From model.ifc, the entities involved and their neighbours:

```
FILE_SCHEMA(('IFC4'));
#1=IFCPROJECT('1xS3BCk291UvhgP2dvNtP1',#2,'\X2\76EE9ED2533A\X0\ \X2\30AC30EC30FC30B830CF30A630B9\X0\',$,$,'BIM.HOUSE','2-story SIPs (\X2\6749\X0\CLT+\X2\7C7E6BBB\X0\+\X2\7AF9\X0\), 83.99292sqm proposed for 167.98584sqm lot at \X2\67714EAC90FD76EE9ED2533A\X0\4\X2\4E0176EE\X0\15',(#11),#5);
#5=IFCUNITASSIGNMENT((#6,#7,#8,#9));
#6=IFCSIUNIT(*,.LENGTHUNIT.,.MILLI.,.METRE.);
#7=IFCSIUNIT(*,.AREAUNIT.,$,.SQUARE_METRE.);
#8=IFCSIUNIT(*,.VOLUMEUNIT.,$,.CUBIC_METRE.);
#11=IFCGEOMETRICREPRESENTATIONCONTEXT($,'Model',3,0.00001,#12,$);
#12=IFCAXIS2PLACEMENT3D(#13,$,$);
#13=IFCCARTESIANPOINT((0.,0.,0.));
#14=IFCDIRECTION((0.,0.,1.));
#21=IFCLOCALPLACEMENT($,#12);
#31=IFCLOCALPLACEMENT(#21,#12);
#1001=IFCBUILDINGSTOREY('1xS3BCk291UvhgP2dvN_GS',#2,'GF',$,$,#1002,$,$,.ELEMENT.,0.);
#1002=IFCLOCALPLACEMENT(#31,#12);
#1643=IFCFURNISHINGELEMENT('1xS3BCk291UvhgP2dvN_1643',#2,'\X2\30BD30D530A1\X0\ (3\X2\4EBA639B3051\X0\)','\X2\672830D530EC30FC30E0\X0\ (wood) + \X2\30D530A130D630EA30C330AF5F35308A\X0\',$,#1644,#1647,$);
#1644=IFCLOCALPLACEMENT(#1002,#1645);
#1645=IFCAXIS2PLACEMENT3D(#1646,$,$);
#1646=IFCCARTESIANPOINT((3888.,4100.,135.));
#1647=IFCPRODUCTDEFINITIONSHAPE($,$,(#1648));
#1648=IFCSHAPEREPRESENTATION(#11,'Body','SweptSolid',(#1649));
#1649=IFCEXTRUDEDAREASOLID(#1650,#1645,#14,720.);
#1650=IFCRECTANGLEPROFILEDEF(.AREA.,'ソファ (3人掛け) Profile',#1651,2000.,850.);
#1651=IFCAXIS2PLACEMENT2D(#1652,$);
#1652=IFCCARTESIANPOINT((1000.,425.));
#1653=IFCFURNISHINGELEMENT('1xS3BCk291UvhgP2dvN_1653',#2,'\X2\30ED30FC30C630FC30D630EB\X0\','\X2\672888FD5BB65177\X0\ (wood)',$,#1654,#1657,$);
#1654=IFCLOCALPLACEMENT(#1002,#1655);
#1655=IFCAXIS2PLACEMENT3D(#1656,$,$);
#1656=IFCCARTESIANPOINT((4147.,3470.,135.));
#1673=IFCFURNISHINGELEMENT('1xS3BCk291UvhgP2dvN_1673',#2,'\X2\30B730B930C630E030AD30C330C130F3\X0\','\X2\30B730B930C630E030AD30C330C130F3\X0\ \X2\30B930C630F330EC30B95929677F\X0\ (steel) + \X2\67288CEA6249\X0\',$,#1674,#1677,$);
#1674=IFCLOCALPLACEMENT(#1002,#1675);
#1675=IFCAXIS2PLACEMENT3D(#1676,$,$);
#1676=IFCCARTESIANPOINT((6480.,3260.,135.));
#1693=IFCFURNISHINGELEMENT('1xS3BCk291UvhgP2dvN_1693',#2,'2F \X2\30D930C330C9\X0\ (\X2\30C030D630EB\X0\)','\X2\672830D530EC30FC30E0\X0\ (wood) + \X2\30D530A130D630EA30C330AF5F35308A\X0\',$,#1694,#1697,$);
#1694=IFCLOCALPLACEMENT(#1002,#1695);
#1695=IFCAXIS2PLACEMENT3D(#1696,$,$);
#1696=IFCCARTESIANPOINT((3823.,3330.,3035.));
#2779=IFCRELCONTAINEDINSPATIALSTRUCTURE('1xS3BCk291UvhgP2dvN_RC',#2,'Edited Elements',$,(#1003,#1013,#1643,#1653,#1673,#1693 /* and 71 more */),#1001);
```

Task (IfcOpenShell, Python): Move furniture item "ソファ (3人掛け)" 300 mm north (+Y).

```python
import ifcopenshell
import ifcopenshell.api.geometry
import ifcopenshell.util.placement
import ifcopenshell.util.unit

model = ifcopenshell.open("model.ifc")
unit_scale = ifcopenshell.util.unit.calculate_unit_scale(model)

item = model.by_guid("1xS3BCk291UvhgP2dvN_1643")
matrix = ifcopenshell.util.placement.get_local_placement(item.ObjectPlacement)
matrix[1, 3] += 0.3 / unit_scale
ifcopenshell.api.geometry.edit_object_placement(model, product=item, matrix=matrix, is_si=False)

print(ifcopenshell.util.placement.get_local_placement(item.ObjectPlacement).round(3) + 0.0)

model.write("model_rev.ifc")
```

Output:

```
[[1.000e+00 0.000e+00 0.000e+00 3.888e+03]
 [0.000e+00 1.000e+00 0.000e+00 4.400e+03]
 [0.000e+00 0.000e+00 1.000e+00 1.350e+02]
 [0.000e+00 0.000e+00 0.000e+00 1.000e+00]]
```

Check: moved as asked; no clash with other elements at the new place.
